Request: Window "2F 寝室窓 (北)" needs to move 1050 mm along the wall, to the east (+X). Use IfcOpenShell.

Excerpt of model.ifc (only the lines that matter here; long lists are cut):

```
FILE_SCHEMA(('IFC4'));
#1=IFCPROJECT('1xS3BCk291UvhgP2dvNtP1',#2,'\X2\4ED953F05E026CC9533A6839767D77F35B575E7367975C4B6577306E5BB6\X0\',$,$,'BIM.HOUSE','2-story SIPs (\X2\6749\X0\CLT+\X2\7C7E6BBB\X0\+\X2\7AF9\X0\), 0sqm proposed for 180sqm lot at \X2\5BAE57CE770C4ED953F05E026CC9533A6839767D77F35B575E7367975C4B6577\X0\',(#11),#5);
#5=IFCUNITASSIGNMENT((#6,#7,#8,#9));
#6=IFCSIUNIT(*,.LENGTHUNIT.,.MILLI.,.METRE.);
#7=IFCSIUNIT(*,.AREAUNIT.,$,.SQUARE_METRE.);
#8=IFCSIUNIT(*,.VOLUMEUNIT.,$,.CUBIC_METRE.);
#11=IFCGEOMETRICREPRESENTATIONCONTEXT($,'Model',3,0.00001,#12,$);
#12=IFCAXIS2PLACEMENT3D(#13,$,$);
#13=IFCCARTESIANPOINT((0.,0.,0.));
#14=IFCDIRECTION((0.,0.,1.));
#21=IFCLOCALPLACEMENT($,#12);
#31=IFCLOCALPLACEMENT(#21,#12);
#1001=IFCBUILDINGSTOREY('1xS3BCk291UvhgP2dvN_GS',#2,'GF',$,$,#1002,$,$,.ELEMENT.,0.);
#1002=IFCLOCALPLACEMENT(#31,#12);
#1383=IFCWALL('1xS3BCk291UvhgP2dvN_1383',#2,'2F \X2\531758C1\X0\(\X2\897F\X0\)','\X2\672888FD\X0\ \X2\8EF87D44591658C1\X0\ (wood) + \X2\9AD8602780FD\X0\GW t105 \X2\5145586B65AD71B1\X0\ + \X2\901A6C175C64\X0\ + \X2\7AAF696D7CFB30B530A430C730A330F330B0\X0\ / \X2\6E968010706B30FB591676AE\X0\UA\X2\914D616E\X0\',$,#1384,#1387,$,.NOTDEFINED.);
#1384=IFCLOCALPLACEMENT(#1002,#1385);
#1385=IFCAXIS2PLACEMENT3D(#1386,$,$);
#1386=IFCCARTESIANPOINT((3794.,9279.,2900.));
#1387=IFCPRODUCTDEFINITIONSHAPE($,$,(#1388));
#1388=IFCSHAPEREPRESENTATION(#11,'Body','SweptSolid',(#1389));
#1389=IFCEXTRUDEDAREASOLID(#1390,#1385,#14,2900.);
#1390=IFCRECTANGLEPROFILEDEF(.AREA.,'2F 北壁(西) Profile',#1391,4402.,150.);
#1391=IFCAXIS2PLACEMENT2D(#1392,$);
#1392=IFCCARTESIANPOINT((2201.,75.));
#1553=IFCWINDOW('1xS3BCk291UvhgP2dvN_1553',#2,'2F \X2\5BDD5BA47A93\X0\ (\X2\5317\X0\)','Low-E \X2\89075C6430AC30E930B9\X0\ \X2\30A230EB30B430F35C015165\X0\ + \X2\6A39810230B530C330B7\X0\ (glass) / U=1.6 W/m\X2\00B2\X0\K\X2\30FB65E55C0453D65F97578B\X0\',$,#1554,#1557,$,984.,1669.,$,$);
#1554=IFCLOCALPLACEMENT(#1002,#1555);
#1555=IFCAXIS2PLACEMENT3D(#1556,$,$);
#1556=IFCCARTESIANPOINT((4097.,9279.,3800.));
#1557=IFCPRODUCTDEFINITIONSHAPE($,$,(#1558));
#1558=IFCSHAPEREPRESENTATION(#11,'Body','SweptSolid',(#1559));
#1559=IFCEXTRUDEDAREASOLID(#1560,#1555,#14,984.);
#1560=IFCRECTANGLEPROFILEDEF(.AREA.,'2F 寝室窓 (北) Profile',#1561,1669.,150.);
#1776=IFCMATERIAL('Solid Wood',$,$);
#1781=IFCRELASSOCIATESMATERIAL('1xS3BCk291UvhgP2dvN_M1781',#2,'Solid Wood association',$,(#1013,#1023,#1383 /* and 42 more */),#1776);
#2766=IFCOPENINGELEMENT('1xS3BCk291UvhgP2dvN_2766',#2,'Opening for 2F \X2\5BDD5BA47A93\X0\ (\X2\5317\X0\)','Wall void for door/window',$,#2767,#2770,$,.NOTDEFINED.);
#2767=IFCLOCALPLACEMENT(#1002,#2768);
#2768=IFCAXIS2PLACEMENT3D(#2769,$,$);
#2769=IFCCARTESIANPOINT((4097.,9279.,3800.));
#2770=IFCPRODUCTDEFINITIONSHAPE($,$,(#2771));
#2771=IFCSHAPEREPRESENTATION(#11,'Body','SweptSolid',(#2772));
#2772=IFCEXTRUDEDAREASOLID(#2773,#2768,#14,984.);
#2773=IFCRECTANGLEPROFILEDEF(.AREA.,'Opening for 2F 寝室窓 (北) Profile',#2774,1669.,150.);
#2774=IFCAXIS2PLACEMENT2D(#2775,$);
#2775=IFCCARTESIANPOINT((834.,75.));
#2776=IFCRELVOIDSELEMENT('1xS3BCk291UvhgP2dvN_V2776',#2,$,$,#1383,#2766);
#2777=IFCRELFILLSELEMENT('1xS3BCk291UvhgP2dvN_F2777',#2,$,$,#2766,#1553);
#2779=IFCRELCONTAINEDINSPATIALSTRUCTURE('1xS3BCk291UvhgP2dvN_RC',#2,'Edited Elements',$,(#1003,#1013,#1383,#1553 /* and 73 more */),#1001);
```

```python
import ifcopenshell
import ifcopenshell.api.geometry
import ifcopenshell.util.placement
import ifcopenshell.util.unit

model = ifcopenshell.open("model.ifc")
unit_scale = ifcopenshell.util.unit.calculate_unit_scale(model)

window = model.by_guid("1xS3BCk291UvhgP2dvN_1553")
opening = window.FillsVoids[0].RelatingOpeningElement
wall = opening.VoidsElements[0].RelatingBuildingElement

wall_matrix = ifcopenshell.util.placement.get_local_placement(wall.ObjectPlacement)
shift = wall_matrix[:3, 0] * 1.05 / unit_scale
before = ifcopenshell.util.placement.get_local_placement(window.ObjectPlacement)[:3, 3].copy()

# The window is not placed relative to its opening, so move both.
for product in (opening, window):
    matrix = ifcopenshell.util.placement.get_local_placement(product.ObjectPlacement)
    matrix[:3, 3] += shift
    ifcopenshell.api.geometry.edit_object_placement(model, product=product, matrix=matrix, is_si=False)

after = ifcopenshell.util.placement.get_local_placement(window.ObjectPlacement)[:3, 3]
print("window moved by", (after - before).round(3) + 0.0)

model.write("model_v2.ifc")
```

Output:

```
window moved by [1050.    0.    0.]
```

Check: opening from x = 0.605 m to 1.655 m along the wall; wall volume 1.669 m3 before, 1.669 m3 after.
